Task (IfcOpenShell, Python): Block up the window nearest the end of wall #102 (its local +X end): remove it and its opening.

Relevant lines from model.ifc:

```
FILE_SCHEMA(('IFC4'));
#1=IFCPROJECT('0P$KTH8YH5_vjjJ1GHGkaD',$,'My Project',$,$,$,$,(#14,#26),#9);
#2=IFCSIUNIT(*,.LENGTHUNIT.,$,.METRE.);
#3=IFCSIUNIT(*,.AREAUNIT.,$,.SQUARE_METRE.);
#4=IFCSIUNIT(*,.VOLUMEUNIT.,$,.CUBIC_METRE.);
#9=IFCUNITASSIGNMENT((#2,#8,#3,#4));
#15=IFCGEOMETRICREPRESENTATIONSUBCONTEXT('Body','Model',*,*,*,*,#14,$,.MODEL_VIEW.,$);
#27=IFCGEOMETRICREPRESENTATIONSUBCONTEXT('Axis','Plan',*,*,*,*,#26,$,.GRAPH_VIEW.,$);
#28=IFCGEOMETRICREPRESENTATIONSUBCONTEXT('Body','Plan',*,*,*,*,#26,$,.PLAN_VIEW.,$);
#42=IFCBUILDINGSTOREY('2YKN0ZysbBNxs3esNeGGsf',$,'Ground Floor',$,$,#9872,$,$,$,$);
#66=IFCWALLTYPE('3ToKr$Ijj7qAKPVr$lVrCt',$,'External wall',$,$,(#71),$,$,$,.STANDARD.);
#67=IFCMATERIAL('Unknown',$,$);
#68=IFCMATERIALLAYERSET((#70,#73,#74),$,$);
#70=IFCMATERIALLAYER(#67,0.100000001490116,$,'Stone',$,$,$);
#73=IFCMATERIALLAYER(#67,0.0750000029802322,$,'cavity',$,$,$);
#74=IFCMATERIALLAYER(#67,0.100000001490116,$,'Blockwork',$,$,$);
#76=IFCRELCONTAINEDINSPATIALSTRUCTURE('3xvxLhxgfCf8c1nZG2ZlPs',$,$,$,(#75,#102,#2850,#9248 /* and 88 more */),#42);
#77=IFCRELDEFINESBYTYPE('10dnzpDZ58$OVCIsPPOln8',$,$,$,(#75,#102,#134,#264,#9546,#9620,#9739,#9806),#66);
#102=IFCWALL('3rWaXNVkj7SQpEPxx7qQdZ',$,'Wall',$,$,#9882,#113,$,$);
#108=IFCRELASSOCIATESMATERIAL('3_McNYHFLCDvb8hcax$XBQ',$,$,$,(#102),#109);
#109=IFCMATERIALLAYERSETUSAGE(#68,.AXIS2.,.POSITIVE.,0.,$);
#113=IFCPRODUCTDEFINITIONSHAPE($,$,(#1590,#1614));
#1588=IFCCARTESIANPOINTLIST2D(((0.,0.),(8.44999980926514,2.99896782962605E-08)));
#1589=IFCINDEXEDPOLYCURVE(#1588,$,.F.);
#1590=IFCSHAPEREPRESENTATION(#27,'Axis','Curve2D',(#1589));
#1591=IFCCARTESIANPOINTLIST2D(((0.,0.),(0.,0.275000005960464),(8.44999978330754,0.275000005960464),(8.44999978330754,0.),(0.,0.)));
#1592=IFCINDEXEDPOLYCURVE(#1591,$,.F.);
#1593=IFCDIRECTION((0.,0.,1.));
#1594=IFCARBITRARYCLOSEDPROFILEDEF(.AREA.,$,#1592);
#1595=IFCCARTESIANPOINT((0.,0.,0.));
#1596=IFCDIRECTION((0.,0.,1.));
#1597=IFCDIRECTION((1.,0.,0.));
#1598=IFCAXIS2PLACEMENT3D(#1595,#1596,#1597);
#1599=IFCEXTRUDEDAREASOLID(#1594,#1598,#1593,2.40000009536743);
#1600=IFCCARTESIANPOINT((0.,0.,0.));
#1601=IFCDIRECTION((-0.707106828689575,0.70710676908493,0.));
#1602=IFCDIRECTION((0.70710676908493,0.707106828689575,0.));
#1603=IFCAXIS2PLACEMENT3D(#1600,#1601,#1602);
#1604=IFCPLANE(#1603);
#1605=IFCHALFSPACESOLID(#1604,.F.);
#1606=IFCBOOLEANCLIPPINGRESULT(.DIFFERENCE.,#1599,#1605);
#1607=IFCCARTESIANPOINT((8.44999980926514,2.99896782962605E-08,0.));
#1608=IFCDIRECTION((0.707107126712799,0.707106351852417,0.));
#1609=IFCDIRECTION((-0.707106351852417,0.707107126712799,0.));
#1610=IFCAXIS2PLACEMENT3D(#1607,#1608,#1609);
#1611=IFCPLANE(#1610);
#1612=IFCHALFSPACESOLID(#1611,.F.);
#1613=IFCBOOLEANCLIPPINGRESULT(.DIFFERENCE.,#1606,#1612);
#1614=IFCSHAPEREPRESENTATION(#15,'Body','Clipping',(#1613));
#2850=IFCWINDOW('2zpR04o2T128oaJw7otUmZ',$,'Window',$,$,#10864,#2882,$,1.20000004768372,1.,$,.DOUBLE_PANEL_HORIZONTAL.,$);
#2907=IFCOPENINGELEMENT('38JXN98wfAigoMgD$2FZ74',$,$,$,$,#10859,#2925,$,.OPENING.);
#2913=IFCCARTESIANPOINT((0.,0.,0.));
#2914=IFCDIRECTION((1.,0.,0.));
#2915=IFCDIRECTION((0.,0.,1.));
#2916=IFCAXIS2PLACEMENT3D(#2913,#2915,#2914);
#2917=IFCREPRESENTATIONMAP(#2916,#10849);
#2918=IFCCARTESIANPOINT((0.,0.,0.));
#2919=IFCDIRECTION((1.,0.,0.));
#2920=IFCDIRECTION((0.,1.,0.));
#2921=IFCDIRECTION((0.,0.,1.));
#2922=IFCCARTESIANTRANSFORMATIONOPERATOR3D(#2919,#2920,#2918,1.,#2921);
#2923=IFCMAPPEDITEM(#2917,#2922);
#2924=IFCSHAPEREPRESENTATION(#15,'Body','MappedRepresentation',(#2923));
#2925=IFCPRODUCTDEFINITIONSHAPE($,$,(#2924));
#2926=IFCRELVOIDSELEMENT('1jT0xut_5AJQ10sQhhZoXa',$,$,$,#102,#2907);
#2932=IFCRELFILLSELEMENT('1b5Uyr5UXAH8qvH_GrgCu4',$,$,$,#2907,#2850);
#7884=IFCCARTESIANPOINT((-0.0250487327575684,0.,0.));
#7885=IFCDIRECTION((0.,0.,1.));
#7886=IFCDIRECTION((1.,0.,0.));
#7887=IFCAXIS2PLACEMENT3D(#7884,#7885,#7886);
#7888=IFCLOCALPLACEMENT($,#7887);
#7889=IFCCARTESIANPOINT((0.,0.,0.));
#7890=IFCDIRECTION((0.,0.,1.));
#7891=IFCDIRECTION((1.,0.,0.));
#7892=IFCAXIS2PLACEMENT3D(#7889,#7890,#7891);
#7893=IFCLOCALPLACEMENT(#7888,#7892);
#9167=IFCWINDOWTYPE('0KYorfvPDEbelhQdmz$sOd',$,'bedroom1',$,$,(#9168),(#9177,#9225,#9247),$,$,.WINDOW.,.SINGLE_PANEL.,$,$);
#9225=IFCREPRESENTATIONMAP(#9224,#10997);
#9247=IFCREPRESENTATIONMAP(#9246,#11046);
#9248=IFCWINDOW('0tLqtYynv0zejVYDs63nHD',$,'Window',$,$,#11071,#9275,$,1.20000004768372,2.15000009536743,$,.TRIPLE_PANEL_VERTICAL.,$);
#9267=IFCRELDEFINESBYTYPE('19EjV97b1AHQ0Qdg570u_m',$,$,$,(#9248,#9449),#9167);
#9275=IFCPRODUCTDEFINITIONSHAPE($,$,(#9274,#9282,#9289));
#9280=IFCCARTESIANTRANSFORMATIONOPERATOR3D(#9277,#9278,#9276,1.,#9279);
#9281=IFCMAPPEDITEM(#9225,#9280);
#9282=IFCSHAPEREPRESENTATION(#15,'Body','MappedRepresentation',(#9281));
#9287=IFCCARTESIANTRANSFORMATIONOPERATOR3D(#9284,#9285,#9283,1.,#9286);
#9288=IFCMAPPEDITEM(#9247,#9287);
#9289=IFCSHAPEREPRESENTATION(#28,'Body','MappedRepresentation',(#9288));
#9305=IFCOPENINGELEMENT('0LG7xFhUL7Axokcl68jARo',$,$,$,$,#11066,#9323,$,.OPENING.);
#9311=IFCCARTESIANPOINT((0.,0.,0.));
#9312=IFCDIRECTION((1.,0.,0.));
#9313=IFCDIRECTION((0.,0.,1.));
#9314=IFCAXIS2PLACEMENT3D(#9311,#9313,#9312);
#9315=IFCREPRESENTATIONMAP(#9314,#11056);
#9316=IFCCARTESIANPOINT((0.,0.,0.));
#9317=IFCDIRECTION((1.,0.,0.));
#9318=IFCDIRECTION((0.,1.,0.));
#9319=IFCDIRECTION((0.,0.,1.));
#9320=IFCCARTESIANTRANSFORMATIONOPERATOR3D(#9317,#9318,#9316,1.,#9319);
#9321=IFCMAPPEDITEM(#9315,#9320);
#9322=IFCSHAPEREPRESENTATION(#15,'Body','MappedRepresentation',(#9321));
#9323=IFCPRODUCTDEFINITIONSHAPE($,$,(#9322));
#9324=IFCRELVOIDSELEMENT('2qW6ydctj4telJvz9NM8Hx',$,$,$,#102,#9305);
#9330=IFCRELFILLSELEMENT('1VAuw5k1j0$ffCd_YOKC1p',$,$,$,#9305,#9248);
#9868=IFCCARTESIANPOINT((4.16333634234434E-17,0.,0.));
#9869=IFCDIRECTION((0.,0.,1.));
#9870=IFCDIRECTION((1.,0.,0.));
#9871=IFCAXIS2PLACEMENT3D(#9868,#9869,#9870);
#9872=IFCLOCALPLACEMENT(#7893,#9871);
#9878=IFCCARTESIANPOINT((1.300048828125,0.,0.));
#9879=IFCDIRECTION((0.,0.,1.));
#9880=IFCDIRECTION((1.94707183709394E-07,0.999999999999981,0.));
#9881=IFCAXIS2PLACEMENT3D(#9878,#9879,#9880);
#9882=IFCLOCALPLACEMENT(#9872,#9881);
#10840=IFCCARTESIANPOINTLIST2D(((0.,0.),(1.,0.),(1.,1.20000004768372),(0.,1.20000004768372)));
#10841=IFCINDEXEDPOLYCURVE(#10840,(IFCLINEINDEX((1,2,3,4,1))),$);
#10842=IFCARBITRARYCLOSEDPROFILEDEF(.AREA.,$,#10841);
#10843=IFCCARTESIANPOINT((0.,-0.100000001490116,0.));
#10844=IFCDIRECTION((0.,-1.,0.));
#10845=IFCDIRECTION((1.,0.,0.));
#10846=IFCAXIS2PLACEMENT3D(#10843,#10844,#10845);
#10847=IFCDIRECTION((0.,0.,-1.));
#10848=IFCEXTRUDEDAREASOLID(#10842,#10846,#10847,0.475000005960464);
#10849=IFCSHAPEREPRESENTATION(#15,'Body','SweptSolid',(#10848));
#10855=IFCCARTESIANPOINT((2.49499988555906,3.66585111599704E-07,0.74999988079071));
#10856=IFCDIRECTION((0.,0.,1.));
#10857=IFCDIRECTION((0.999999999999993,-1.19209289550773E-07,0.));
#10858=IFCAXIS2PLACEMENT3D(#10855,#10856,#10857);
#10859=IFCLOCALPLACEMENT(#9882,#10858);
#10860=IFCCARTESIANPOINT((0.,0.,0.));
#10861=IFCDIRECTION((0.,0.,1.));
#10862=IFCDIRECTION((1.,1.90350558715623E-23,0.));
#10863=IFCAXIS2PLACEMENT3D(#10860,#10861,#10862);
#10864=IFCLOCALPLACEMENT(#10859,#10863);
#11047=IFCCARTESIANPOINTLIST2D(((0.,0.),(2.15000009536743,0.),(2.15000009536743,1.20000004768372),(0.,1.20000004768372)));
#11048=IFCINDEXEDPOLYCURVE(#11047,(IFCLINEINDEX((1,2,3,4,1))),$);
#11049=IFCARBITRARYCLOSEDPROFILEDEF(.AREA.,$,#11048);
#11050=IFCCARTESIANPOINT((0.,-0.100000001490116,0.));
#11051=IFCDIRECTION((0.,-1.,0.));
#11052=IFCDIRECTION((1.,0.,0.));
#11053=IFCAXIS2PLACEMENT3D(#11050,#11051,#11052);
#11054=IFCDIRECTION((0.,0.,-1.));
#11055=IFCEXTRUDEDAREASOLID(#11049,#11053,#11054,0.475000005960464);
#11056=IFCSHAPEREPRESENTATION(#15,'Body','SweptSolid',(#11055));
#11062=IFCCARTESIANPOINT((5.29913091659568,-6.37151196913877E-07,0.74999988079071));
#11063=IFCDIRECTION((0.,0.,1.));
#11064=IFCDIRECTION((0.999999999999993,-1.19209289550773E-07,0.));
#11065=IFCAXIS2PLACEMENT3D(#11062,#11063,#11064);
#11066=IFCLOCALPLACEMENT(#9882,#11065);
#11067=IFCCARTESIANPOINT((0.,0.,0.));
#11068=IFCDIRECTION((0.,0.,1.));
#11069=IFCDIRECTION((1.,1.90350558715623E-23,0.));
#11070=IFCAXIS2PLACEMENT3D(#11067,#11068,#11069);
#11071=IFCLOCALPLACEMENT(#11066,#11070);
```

```python
import ifcopenshell
import ifcopenshell.api.feature
import ifcopenshell.api.root
import ifcopenshell.geom
import ifcopenshell.util.shape

model = ifcopenshell.open("model.ifc")
settings = ifcopenshell.geom.settings()


def volume(element):
    """Net volume in cubic metres, openings subtracted."""
    shape = ifcopenshell.geom.create_shape(settings, element)
    return ifcopenshell.util.shape.get_volume(shape.geometry)


window = model.by_guid("0tLqtYynv0zejVYDs63nHD")
opening = window.FillsVoids[0].RelatingOpeningElement
wall = opening.VoidsElements[0].RelatingBuildingElement
before = volume(wall)

ifcopenshell.api.root.remove_product(model, product=window)
ifcopenshell.api.feature.remove_feature(model, feature=opening)

after = volume(wall)

print(f"wall volume {before:.3f} -> {after:.3f} m3")

model.write("model_updated.ifc")
```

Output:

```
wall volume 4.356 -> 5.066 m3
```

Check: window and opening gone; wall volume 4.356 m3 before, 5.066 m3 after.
